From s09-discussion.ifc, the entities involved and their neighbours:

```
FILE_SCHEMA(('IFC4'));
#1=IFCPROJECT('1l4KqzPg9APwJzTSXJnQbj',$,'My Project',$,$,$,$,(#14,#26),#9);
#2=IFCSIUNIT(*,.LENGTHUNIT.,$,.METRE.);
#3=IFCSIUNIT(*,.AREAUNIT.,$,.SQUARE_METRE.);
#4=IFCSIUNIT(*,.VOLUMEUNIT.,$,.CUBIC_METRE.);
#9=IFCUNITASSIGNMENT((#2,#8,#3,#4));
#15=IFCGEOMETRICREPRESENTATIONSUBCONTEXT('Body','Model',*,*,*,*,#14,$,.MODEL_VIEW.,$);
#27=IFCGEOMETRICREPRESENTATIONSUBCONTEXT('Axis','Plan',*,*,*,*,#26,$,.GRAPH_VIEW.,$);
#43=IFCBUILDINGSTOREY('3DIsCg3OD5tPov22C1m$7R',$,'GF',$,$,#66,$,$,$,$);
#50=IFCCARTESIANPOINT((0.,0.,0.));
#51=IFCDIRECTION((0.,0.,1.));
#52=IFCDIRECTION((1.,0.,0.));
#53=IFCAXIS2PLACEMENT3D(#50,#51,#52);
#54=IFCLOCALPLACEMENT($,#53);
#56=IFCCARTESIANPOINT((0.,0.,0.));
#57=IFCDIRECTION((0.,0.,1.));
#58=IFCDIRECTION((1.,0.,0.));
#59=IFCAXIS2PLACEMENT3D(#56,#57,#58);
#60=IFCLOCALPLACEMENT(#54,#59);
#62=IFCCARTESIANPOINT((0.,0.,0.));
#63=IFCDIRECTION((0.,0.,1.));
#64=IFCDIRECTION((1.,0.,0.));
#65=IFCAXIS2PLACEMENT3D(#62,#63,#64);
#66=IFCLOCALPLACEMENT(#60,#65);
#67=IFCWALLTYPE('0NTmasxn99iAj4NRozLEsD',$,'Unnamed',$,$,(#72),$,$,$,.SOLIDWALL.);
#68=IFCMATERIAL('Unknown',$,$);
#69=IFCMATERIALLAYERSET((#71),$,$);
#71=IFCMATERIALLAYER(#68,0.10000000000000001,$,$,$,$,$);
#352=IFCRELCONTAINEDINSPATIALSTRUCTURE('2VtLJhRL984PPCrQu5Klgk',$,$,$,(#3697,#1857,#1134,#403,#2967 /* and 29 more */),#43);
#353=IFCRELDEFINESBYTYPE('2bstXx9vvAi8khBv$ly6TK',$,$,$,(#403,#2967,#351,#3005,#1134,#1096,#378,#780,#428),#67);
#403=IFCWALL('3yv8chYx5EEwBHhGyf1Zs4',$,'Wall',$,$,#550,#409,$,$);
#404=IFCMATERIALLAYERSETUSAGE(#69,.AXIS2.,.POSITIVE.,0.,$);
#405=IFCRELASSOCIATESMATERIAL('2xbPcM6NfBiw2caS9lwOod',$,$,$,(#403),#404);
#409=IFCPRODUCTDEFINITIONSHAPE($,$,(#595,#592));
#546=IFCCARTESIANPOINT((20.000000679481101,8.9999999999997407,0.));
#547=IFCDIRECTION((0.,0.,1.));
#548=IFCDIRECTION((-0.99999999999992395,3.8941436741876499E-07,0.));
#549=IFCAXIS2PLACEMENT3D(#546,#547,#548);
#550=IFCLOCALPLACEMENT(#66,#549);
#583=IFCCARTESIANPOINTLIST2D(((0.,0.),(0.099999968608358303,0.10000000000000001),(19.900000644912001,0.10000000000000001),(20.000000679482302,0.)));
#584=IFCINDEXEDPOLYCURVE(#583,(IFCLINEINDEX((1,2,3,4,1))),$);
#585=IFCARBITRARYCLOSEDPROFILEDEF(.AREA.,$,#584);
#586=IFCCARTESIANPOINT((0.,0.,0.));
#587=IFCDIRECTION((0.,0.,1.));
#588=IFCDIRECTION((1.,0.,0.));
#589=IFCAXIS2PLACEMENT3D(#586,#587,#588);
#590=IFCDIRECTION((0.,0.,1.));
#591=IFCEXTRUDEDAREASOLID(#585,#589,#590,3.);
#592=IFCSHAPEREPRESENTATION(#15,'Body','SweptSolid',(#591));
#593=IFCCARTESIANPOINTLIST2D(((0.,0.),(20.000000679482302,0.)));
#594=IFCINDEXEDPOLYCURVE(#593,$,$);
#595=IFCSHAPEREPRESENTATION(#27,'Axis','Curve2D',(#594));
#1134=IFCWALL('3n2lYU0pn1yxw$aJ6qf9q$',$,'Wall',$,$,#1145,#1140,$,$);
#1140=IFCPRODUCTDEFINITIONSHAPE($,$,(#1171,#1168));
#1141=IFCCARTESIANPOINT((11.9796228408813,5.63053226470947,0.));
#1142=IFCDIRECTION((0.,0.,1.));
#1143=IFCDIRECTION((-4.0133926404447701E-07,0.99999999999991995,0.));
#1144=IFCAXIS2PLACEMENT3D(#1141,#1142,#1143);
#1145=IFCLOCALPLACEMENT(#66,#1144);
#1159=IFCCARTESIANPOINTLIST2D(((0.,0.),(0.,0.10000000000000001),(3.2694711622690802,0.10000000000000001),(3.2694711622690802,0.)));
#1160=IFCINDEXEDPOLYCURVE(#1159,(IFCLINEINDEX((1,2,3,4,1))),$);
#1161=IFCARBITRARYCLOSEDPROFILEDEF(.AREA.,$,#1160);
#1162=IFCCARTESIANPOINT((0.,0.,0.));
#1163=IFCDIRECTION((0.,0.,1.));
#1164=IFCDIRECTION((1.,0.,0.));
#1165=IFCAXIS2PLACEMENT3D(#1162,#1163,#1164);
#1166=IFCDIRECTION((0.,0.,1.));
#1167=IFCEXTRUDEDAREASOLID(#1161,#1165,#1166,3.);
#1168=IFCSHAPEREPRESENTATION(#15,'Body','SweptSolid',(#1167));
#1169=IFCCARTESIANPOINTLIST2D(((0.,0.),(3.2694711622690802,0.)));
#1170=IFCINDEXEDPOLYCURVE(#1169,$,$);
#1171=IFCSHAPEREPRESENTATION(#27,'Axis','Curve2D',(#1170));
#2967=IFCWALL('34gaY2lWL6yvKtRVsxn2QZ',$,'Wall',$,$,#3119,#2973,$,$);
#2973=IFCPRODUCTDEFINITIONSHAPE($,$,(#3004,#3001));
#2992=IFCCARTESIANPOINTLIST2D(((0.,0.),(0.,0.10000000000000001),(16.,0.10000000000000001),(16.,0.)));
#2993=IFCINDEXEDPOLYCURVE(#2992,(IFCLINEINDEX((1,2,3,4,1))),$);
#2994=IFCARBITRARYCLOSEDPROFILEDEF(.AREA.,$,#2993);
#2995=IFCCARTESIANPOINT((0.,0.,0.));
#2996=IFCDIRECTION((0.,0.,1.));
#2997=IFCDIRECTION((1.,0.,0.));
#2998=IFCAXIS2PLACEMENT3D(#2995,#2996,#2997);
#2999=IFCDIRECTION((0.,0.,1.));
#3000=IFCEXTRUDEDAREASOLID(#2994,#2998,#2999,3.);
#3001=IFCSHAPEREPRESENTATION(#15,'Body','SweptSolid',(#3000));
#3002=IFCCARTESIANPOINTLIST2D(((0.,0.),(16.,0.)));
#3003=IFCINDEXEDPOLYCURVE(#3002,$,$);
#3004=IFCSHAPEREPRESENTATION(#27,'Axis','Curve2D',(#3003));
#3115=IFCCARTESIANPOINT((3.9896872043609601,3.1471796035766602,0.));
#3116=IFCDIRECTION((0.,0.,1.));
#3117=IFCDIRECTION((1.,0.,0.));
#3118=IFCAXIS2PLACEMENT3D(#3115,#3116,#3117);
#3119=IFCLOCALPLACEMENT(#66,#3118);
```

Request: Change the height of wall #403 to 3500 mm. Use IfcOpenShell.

```python
import ifcopenshell
import ifcopenshell.geom
import ifcopenshell.util.representation
import ifcopenshell.util.shape

model = ifcopenshell.open("s09-discussion.ifc")
settings = ifcopenshell.geom.settings()


def volume(element):
    """Net volume in cubic metres, openings subtracted."""
    shape = ifcopenshell.geom.create_shape(settings, element)
    return ifcopenshell.util.shape.get_volume(shape.geometry)


wall = model.by_guid("3yv8chYx5EEwBHhGyf1Zs4")
before = volume(wall)

body = ifcopenshell.util.representation.get_representation(wall, "Model", "Body")
solid = body.Items[0]
old_height = solid.Depth
solid.Depth = 3.5
after = volume(wall)

print(f"height {old_height:g} -> {solid.Depth:g}, volume {before:.3f} -> {after:.3f} m3")

model.write("s09-discussion_rev.ifc")
```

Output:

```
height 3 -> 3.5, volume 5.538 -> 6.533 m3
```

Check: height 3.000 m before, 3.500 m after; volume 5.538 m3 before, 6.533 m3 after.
